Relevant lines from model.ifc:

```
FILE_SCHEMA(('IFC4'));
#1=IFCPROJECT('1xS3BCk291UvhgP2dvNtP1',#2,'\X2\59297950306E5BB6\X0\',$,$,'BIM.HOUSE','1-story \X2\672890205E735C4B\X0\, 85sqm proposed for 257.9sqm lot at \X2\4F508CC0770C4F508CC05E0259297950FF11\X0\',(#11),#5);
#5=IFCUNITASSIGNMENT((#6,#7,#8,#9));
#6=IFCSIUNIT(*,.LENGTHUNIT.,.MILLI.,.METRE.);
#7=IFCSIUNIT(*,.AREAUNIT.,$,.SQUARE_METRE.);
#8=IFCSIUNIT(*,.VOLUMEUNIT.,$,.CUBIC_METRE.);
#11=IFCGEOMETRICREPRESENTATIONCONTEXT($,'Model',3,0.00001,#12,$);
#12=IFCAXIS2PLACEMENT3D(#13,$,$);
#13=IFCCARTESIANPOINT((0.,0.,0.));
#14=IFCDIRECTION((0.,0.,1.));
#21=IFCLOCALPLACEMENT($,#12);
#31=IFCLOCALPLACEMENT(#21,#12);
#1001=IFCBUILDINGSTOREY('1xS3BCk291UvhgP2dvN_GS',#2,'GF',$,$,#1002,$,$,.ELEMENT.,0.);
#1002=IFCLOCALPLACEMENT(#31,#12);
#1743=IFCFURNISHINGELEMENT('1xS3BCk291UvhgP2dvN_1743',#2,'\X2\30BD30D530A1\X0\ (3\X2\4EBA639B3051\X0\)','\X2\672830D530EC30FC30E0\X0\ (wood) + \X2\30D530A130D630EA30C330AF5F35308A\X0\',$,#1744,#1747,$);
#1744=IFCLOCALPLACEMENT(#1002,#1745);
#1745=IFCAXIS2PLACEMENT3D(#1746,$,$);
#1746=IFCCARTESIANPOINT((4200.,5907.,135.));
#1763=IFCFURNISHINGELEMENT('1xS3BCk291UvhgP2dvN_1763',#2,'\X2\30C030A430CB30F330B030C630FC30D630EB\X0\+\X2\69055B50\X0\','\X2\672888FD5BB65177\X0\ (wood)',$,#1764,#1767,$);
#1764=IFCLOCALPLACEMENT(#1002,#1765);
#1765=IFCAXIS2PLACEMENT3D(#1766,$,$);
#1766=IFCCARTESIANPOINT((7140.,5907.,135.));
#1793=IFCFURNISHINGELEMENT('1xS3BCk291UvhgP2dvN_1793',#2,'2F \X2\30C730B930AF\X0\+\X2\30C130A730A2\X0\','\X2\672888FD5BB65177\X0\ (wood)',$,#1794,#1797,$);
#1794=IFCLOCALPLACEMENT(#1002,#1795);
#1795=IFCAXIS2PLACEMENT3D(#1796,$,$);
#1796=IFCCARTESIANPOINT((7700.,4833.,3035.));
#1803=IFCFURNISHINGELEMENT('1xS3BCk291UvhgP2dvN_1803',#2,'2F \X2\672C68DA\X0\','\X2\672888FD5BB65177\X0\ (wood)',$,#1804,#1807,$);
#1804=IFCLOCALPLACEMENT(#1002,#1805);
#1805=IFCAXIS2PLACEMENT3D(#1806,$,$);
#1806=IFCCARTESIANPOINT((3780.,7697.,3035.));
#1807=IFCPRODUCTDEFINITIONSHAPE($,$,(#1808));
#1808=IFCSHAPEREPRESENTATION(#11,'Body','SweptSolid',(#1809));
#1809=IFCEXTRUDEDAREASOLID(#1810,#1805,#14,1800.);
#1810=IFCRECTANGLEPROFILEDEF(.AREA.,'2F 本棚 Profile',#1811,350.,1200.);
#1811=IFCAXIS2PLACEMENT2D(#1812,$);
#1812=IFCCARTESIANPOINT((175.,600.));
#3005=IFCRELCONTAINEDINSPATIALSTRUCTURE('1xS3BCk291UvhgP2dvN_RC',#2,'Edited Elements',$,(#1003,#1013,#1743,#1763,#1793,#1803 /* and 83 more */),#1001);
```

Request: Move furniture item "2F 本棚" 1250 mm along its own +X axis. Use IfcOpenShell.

```python
import ifcopenshell
import ifcopenshell.api.geometry
import ifcopenshell.util.placement

model = ifcopenshell.open("model.ifc")

item = model.by_guid("1xS3BCk291UvhgP2dvN_1803")
matrix = ifcopenshell.util.placement.get_local_placement(item.ObjectPlacement)
matrix[:3, 3] += matrix[:3, 0] * 1250.0
ifcopenshell.api.geometry.edit_object_placement(model, product=item, matrix=matrix, is_si=False)

print(ifcopenshell.util.placement.get_local_placement(item.ObjectPlacement).round(3) + 0.0)

model.write("model_rev.ifc")
```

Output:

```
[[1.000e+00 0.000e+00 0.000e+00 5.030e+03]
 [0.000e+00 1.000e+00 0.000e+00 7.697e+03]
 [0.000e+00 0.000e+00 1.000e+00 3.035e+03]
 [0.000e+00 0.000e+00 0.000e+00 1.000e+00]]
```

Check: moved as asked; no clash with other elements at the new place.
